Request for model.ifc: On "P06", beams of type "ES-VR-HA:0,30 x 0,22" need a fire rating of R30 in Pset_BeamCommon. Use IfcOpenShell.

First a look at what the model holds.

```python
import ifcopenshell
import ifcopenshell.util.element

model = ifcopenshell.open("model.ifc")
print(model.schema)
storey = next(s for s in model.by_type("IfcBuildingStorey") if s.Name == "P06")
beams = [e for e in ifcopenshell.util.element.get_decomposition(storey) if e.is_a("IfcBeam")]
seen = {}
for e in beams:
    element_type = ifcopenshell.util.element.get_type(e)
    key = (element_type.Name if element_type != e and element_type else None, ifcopenshell.util.element.get_pset(e, "Pset_BeamCommon", "FireRating"))
    seen[key] = seen.get(key, 0) + 1
for (name, value), count in sorted(seen.items(), key=str):
    print(count, "x", name, "|", value)
```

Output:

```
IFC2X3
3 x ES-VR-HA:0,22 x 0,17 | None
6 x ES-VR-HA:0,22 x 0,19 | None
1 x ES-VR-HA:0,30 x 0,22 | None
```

```python
import ifcopenshell
import ifcopenshell.api.pset
import ifcopenshell.util.element

model = ifcopenshell.open("model.ifc")

storey = next(s for s in model.by_type("IfcBuildingStorey") if s.Name == "P06")
beams = [e for e in ifcopenshell.util.element.get_decomposition(storey) if e.is_a("IfcBeam")]

count = 0
for e in beams:
    element_type = ifcopenshell.util.element.get_type(e)
    if element_type in (None, e) or element_type.Name != "ES-VR-HA:0,30 x 0,22":
        continue
    # add_pset returns the element's existing set when there is one.
    pset = ifcopenshell.api.pset.add_pset(model, product=e, name="Pset_BeamCommon")
    ifcopenshell.api.pset.edit_pset(model, pset=pset, properties={"FireRating": "R30"})
    count += 1

print(count, "beams updated")

model.write("model_updated.ifc")
```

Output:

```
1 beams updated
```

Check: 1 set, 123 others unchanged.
